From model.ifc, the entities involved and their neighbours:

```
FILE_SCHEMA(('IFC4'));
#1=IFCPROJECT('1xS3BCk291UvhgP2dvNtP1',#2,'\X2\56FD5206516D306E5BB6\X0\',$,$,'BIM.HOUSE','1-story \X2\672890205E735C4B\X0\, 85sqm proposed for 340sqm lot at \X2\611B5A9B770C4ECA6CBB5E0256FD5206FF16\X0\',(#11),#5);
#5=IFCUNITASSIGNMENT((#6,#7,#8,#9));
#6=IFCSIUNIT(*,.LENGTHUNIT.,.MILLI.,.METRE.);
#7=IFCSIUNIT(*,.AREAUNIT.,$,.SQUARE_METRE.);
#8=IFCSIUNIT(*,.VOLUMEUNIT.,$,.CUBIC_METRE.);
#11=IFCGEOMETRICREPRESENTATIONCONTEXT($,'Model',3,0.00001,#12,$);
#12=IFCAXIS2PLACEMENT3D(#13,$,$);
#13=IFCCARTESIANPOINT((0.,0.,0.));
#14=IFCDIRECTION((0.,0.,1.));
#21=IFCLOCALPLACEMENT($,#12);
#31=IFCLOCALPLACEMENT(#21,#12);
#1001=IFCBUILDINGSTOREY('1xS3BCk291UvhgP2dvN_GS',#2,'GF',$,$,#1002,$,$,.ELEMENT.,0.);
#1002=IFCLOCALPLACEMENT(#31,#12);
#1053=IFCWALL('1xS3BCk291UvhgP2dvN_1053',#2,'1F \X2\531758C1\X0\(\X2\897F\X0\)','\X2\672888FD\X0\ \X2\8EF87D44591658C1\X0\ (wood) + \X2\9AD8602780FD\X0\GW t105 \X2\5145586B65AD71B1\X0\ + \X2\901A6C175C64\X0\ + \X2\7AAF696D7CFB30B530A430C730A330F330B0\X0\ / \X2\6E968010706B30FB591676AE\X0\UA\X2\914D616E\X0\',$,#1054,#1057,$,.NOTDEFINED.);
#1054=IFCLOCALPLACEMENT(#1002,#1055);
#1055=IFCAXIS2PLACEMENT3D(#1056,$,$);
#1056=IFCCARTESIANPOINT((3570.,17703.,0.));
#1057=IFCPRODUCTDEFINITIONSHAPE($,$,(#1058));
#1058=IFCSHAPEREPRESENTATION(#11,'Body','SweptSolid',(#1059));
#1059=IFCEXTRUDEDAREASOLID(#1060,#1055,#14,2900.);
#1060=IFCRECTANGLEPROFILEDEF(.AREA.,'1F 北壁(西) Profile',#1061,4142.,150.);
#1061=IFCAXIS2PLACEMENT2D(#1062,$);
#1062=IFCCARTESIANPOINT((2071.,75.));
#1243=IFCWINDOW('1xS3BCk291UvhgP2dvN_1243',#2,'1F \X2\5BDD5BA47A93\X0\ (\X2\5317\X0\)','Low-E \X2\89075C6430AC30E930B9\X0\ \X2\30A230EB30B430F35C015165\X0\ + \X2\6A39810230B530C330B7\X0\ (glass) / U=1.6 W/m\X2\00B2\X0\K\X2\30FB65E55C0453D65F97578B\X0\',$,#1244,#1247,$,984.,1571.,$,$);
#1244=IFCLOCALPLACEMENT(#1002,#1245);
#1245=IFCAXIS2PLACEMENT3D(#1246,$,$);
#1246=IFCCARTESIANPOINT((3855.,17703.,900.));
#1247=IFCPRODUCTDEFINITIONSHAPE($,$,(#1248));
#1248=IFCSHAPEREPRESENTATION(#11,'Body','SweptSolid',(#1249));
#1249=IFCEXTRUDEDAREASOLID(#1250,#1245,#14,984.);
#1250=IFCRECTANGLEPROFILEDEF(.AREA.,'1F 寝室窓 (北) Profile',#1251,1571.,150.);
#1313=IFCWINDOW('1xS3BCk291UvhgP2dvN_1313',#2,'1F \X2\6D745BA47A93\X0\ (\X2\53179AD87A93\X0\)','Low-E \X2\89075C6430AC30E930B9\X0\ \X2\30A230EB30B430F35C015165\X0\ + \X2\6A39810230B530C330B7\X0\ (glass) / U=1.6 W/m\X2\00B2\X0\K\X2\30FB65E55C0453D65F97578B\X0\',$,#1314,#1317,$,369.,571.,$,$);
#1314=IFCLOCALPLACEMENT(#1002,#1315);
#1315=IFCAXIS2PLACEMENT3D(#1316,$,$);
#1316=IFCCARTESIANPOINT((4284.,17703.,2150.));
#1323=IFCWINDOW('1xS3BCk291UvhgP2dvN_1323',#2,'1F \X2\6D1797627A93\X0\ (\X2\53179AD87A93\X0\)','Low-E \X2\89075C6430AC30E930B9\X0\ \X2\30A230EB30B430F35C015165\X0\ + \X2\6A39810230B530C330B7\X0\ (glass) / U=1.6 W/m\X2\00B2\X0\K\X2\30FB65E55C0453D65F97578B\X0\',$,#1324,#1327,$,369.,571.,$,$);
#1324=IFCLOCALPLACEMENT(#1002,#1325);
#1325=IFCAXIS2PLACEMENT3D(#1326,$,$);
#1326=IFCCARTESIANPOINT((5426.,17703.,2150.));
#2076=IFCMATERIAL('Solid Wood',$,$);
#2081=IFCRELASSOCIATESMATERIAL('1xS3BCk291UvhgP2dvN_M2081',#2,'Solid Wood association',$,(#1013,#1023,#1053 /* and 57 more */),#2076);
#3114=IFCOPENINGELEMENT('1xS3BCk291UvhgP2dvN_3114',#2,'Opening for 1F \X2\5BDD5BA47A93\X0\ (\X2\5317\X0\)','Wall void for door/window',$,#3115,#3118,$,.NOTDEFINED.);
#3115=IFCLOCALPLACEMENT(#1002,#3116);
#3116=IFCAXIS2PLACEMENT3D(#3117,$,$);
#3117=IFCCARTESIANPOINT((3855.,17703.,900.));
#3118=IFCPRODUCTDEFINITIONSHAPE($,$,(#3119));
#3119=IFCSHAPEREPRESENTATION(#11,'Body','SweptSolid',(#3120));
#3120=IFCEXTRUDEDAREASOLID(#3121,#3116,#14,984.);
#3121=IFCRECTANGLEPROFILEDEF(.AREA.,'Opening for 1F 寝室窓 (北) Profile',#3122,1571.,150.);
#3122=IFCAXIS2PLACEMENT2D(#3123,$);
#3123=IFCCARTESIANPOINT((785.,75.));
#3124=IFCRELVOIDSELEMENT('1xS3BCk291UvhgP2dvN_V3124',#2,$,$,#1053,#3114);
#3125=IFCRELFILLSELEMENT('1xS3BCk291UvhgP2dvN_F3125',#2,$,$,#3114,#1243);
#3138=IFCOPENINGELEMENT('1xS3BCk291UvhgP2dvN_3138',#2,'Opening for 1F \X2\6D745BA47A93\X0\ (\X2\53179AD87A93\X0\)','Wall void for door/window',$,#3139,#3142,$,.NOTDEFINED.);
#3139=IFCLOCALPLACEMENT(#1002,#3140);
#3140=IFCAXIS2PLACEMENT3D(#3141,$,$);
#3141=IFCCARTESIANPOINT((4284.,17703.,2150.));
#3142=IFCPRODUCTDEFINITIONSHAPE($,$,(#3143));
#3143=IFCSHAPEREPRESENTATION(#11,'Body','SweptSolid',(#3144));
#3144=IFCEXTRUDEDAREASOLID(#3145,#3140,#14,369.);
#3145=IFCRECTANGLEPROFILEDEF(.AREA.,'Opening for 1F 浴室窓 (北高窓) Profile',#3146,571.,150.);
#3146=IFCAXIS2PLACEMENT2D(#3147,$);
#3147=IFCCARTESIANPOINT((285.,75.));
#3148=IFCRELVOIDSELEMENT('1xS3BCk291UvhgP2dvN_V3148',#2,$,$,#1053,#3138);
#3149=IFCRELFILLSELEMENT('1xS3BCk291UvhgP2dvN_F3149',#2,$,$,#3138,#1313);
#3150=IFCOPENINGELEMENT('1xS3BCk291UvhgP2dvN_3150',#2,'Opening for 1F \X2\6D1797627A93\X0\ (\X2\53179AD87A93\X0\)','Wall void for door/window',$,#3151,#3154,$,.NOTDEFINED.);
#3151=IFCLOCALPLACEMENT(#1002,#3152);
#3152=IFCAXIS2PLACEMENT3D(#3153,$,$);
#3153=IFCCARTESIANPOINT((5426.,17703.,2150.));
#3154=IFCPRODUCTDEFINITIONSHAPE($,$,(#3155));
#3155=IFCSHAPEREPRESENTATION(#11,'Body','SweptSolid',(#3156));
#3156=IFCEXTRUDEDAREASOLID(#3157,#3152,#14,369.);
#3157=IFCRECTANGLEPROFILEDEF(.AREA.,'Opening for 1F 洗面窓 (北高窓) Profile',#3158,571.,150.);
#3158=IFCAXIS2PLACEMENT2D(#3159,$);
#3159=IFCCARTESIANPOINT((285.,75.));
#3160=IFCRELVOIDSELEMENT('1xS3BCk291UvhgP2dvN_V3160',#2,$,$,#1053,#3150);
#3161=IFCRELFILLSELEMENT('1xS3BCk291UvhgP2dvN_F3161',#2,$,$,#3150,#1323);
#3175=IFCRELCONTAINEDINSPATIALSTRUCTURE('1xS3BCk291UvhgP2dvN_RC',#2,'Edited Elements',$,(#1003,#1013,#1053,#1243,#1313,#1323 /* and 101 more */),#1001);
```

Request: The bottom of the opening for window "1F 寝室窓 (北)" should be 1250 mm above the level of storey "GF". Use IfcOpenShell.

```python
import numpy as np
import ifcopenshell
import ifcopenshell.api.geometry
import ifcopenshell.geom
import ifcopenshell.util.element
import ifcopenshell.util.placement
import ifcopenshell.util.shape
import ifcopenshell.util.unit

model = ifcopenshell.open("model.ifc")
unit_scale = ifcopenshell.util.unit.calculate_unit_scale(model)

window = model.by_guid("1xS3BCk291UvhgP2dvN_1243")
opening = window.FillsVoids[0].RelatingOpeningElement
storey = ifcopenshell.util.element.get_container(window, ifc_class="IfcBuildingStorey")
level = ifcopenshell.util.placement.get_local_placement(storey.ObjectPlacement)[2, 3]

# The opening's origin need not be at the sill, so measure its lowest point.
shape = ifcopenshell.geom.create_shape(ifcopenshell.geom.settings(), opening)
bottom = ifcopenshell.util.shape.get_shape_bottom_elevation(shape, shape.geometry) / unit_scale
dz = level + 1.25 / unit_scale - bottom

shift = np.array([0.0, 0.0, dz])
# The window is not placed relative to its opening, so move both.
for product in (opening, window):
    matrix = ifcopenshell.util.placement.get_local_placement(product.ObjectPlacement)
    matrix[:3, 3] += shift
    ifcopenshell.api.geometry.edit_object_placement(model, product=product, matrix=matrix, is_si=False)

print(f"moved by {dz * unit_scale:+.3f} m")

model.write("model_edited.ifc")
```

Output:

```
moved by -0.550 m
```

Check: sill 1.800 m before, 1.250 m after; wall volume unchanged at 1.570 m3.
